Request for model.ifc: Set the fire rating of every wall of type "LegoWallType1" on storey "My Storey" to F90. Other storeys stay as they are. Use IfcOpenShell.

First a look at what the model holds.

```python
import ifcopenshell
import ifcopenshell.util.element

model = ifcopenshell.open("model.ifc")
print(model.schema)
storey = next(s for s in model.by_type("IfcBuildingStorey") if s.Name == "My Storey")
walls = [e for e in ifcopenshell.util.element.get_decomposition(storey) if e.is_a("IfcWall")]
seen = {}
for e in walls:
    element_type = ifcopenshell.util.element.get_type(e)
    key = (element_type.Name if element_type != e and element_type else None, ifcopenshell.util.element.get_pset(e, "Pset_WallCommon", "FireRating"))
    seen[key] = seen.get(key, 0) + 1
for (name, value), count in sorted(seen.items(), key=str):
    print(count, "x", name, "|", value)
```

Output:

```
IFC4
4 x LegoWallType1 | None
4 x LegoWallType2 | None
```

```python
import ifcopenshell
import ifcopenshell.api.pset
import ifcopenshell.util.element

model = ifcopenshell.open("model.ifc")

storey = next(s for s in model.by_type("IfcBuildingStorey") if s.Name == "My Storey")
walls = [e for e in ifcopenshell.util.element.get_decomposition(storey) if e.is_a("IfcWall")]

count = 0
for e in walls:
    element_type = ifcopenshell.util.element.get_type(e)
    if element_type in (None, e) or element_type.Name != "LegoWallType1":
        continue
    # add_pset returns the element's existing set when there is one.
    pset = ifcopenshell.api.pset.add_pset(model, product=e, name="Pset_WallCommon")
    ifcopenshell.api.pset.edit_pset(model, pset=pset, properties={"FireRating": "F90"})
    count += 1

print(count, "walls updated")

model.write("model_edited.ifc")
```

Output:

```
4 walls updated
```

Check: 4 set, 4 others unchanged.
